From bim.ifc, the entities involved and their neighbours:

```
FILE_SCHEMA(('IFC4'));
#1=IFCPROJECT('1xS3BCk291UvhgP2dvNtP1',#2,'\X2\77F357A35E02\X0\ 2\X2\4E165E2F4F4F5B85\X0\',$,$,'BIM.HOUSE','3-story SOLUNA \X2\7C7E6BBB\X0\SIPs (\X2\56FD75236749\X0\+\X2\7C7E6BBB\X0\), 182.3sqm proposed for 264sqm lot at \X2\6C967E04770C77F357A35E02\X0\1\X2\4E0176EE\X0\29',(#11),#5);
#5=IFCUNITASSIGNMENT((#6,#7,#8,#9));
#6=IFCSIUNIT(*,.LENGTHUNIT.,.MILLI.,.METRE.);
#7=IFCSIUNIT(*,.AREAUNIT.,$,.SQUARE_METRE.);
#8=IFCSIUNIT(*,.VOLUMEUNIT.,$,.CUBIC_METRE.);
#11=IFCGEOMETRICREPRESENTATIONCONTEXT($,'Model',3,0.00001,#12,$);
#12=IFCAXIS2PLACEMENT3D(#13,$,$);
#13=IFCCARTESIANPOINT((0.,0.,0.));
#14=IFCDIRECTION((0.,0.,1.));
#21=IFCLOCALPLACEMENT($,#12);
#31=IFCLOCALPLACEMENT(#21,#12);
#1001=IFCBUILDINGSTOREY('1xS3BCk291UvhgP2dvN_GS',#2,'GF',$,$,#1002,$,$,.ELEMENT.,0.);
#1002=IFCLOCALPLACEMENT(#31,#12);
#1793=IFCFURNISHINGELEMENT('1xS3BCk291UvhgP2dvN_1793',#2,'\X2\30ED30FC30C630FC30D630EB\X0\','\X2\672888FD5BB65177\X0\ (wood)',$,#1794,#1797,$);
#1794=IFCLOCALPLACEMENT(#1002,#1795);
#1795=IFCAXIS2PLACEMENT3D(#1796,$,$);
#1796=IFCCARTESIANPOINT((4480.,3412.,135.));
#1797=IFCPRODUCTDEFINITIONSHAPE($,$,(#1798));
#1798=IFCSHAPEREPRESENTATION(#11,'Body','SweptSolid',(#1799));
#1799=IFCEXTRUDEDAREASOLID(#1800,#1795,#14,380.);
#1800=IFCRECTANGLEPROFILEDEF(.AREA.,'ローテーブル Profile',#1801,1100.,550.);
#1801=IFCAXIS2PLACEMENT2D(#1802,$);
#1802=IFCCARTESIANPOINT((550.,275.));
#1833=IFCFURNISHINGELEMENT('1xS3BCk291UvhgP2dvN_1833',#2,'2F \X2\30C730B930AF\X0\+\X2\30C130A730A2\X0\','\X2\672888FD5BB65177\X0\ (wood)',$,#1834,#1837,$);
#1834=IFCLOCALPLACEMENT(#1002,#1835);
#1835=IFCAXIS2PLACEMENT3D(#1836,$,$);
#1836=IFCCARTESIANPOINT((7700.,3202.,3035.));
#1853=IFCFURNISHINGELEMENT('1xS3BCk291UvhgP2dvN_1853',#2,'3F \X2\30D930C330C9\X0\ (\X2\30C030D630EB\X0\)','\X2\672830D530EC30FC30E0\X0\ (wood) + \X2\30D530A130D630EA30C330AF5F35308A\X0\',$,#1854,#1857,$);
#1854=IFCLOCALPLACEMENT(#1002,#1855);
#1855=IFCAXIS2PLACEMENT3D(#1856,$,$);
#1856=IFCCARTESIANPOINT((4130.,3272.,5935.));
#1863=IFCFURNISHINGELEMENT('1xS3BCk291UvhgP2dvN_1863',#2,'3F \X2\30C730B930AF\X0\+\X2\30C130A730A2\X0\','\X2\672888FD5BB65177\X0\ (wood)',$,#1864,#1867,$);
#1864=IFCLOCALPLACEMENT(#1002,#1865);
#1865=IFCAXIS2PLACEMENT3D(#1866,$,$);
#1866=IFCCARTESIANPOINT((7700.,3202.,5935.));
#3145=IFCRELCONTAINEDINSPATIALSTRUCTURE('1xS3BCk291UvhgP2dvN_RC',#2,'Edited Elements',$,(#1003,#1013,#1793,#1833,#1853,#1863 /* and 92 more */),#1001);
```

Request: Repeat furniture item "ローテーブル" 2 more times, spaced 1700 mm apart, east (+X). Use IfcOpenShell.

```python
import numpy as np
import ifcopenshell
import ifcopenshell.api.geometry
import ifcopenshell.api.root
import ifcopenshell.util.element
import ifcopenshell.util.placement
import ifcopenshell.util.unit

model = ifcopenshell.open("bim.ifc")
unit_scale = ifcopenshell.util.unit.calculate_unit_scale(model)


def reuse_history(source, copy):
    """copy_class also copies each property set's owner history, people and application; keep the originals."""
    for rel in copy.IsDefinedBy:
        if rel.is_a("IfcRelDefinesByProperties") and (history := rel.RelatingPropertyDefinition.OwnerHistory):
            rel.RelatingPropertyDefinition.OwnerHistory = source.OwnerHistory
            ifcopenshell.util.element.remove_deep2(model, history)


source = model.by_guid("1xS3BCk291UvhgP2dvN_1793")
base = ifcopenshell.util.placement.get_local_placement(source.ObjectPlacement)
step = np.array([1.0, 0.0, 0.0]) * 1.7 / unit_scale

for i in range(1, 3):
    copy = ifcopenshell.api.root.copy_class(model, product=source)
    copy.Representation = ifcopenshell.util.element.copy_deep(
        model, source.Representation, exclude=["IfcGeometricRepresentationContext", "IfcRepresentationMap"]
    )
    reuse_history(source, copy)
    matrix = base.copy()
    matrix[:3, 3] += i * step
    print("added at", matrix[:3, 3].round(3) + 0.0)
    ifcopenshell.api.geometry.edit_object_placement(model, product=copy, matrix=matrix, is_si=False)

model.write("bim_v2.ifc")
```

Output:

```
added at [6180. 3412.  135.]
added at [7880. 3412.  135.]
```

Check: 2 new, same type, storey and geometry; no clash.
